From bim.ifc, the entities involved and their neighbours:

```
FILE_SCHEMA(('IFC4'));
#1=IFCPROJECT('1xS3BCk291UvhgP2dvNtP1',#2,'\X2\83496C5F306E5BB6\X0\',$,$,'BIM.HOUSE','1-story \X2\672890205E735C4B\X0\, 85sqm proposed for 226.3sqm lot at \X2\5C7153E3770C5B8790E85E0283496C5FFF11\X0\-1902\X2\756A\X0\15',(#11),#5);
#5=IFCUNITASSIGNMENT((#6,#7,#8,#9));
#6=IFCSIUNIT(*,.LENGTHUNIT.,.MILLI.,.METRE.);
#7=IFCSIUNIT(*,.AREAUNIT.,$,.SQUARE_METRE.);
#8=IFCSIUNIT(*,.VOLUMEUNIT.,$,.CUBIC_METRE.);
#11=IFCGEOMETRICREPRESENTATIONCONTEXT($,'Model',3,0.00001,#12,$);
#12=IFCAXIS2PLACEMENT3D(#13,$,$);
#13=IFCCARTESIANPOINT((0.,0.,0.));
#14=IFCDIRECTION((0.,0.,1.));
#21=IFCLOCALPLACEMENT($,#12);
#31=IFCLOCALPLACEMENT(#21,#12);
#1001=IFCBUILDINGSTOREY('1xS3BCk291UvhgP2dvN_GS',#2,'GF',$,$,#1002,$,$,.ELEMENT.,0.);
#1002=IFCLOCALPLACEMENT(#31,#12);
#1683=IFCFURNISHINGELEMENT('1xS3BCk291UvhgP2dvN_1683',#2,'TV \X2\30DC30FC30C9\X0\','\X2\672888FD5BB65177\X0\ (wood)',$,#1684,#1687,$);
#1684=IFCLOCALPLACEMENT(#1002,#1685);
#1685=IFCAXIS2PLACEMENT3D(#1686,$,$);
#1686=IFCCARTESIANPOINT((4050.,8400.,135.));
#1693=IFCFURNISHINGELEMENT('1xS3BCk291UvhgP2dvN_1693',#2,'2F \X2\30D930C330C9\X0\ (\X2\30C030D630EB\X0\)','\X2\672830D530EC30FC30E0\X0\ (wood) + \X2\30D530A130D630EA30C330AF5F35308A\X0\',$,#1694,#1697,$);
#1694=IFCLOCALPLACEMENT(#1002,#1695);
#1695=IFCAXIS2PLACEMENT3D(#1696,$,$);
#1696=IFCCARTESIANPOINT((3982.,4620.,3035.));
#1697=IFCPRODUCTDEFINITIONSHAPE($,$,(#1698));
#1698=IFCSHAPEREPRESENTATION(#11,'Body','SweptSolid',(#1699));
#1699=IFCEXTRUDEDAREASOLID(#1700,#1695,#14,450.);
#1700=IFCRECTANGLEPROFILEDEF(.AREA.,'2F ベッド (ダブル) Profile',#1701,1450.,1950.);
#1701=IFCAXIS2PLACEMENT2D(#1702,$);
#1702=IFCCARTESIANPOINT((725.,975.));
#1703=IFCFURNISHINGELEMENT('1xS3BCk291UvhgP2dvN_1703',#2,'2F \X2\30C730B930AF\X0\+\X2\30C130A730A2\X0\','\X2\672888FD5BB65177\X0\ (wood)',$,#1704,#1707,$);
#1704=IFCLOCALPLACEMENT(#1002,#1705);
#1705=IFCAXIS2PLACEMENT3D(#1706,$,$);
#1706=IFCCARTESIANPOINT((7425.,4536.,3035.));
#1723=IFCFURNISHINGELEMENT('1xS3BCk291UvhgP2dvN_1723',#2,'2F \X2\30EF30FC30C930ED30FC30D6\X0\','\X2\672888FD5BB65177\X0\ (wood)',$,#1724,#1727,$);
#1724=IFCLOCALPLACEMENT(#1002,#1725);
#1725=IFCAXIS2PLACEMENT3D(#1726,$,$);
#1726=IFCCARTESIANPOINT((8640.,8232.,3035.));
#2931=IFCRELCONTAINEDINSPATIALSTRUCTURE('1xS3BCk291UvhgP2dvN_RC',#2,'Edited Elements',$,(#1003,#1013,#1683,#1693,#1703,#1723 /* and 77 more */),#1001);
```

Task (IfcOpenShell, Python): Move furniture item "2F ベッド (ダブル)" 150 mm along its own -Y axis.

```python
import ifcopenshell
import ifcopenshell.api.geometry
import ifcopenshell.util.placement
import ifcopenshell.util.unit

model = ifcopenshell.open("bim.ifc")
unit_scale = ifcopenshell.util.unit.calculate_unit_scale(model)

item = model.by_id(1693)
matrix = ifcopenshell.util.placement.get_local_placement(item.ObjectPlacement)
matrix[:3, 3] -= matrix[:3, 1] * 0.15 / unit_scale
ifcopenshell.api.geometry.edit_object_placement(model, product=item, matrix=matrix, is_si=False)

print(ifcopenshell.util.placement.get_local_placement(item.ObjectPlacement).round(3) + 0.0)

model.write("bim-out.ifc")
```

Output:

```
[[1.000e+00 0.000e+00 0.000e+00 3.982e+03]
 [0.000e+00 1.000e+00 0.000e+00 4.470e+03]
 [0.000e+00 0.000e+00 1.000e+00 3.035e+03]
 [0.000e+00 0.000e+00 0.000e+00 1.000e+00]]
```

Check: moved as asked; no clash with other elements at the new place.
